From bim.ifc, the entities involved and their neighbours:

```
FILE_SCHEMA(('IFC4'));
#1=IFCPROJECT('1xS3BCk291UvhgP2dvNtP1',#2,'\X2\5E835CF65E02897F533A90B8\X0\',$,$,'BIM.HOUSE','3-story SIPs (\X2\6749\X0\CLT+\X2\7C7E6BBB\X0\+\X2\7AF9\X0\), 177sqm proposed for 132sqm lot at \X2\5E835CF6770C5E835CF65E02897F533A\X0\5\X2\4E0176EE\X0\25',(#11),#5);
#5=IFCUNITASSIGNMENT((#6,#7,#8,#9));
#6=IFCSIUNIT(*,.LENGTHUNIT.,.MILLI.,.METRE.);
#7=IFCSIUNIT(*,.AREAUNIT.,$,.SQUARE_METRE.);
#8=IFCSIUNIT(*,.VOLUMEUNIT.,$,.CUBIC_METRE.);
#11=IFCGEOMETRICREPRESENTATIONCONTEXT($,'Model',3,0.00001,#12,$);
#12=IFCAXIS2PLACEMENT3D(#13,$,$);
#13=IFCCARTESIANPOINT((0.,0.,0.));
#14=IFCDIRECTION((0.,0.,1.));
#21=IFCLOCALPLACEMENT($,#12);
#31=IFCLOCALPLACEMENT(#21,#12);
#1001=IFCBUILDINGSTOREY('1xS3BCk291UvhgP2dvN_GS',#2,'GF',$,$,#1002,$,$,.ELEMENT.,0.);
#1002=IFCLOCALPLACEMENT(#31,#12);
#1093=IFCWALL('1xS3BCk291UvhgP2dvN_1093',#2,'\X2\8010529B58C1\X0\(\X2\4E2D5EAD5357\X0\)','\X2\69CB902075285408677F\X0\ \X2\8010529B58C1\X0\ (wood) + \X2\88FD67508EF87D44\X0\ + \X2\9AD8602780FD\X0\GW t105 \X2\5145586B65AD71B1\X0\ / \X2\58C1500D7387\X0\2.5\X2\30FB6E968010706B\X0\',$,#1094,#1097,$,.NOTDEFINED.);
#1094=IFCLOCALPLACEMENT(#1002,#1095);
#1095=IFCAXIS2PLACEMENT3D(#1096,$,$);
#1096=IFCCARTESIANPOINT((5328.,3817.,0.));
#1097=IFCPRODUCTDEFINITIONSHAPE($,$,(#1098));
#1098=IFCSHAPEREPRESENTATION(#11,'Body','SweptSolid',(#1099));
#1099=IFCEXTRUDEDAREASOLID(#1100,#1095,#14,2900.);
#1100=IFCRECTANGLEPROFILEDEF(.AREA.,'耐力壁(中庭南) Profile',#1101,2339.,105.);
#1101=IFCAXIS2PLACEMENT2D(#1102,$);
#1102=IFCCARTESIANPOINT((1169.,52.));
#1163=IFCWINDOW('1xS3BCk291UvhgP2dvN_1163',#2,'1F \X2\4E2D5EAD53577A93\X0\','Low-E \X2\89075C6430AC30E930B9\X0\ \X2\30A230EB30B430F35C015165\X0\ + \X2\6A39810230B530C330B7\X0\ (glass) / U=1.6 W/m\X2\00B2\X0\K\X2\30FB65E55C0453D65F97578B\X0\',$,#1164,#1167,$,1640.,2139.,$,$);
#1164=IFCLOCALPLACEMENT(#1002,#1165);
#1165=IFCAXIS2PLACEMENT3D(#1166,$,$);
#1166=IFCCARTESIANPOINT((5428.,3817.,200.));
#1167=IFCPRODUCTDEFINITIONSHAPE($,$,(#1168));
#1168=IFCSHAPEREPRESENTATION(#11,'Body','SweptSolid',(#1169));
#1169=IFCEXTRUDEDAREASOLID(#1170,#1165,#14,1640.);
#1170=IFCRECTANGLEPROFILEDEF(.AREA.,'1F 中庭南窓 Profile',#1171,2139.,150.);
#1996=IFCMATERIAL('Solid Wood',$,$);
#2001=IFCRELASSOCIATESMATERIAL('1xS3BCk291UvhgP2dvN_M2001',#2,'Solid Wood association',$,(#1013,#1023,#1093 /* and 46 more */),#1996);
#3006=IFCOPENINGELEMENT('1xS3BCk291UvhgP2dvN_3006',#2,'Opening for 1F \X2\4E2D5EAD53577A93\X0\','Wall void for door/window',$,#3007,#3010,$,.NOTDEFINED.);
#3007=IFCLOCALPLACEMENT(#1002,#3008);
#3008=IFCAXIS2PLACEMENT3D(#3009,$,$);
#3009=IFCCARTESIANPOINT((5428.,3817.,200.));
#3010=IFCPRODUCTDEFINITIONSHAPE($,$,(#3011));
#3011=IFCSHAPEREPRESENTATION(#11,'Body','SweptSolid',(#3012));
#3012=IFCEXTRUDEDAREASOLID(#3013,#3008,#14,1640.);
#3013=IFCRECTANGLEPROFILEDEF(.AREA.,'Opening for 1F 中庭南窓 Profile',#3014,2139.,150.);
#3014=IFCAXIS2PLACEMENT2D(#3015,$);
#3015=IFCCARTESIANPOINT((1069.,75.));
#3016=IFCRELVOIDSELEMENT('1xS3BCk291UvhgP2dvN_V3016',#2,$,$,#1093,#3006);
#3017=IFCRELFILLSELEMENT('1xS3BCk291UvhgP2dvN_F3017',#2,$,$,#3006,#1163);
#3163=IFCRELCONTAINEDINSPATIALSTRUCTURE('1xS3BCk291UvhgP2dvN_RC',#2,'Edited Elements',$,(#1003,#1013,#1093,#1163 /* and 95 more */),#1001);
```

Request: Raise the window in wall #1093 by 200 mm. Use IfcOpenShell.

```python
import numpy as np
import ifcopenshell
import ifcopenshell.api.geometry
import ifcopenshell.util.placement
import ifcopenshell.util.unit

model = ifcopenshell.open("bim.ifc")
unit_scale = ifcopenshell.util.unit.calculate_unit_scale(model)

window = model.by_guid("1xS3BCk291UvhgP2dvN_1163")
opening = window.FillsVoids[0].RelatingOpeningElement
dz = 200.0

shift = np.array([0.0, 0.0, dz])
# The window is not placed relative to its opening, so move both.
for product in (opening, window):
    matrix = ifcopenshell.util.placement.get_local_placement(product.ObjectPlacement)
    matrix[:3, 3] += shift
    ifcopenshell.api.geometry.edit_object_placement(model, product=product, matrix=matrix, is_si=False)

print(f"moved by {dz * unit_scale:+.3f} m")

model.write("bim_v2.ifc")
```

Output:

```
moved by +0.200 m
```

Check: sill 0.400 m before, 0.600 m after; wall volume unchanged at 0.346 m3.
